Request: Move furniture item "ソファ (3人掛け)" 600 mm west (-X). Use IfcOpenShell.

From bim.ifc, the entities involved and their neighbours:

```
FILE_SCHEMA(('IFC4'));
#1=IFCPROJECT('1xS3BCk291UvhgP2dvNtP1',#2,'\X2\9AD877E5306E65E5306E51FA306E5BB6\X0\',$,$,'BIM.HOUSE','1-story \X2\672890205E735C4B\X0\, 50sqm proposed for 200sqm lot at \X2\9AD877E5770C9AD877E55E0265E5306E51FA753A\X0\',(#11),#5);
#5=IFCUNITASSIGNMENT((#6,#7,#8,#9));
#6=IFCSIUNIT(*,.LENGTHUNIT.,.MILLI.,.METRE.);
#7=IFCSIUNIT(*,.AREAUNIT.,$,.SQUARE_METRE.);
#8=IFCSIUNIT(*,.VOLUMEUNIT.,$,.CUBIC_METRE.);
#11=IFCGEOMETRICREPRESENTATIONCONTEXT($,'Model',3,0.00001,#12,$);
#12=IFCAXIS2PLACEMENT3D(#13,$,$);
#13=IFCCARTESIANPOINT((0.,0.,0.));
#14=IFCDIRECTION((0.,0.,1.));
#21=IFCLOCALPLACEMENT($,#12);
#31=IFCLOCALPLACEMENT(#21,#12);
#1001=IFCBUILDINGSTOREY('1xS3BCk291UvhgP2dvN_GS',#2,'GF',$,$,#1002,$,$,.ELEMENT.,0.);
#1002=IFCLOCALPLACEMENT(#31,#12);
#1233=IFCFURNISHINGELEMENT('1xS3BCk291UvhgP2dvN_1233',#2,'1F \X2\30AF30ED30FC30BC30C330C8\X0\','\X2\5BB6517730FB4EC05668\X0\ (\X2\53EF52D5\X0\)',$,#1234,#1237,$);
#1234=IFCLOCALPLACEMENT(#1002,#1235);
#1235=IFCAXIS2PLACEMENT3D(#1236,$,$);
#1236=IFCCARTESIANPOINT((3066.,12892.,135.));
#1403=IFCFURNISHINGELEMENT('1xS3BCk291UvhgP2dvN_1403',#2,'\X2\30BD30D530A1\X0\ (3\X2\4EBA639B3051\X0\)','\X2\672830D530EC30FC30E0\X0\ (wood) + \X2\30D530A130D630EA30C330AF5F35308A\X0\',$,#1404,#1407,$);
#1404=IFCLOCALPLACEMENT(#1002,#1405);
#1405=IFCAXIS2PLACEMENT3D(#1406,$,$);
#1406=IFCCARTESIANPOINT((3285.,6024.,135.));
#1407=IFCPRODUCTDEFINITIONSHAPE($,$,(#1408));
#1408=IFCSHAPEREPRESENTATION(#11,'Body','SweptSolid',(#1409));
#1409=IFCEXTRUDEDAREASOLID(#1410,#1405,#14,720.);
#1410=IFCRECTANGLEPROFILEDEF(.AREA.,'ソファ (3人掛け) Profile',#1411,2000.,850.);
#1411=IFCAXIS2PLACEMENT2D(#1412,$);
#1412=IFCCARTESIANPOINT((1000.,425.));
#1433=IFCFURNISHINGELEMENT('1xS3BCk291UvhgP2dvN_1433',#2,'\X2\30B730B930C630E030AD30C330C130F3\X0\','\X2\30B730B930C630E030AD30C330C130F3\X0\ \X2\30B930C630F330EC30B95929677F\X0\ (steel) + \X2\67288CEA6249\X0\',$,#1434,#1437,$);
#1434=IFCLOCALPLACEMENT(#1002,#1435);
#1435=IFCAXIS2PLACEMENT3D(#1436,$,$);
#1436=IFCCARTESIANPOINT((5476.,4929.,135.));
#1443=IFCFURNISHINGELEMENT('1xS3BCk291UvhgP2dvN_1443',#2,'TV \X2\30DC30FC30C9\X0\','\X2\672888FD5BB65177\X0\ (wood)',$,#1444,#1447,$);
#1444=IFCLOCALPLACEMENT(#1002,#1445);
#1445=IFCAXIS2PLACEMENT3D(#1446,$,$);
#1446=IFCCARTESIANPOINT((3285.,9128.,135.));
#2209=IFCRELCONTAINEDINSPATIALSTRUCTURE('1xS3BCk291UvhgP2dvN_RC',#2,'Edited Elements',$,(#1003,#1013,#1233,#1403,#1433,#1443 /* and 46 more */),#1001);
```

```python
import ifcopenshell
import ifcopenshell.api.geometry
import ifcopenshell.util.placement
import ifcopenshell.util.unit

model = ifcopenshell.open("bim.ifc")
unit_scale = ifcopenshell.util.unit.calculate_unit_scale(model)

item = model.by_id(1403)
matrix = ifcopenshell.util.placement.get_local_placement(item.ObjectPlacement)
matrix[0, 3] -= 0.6 / unit_scale
ifcopenshell.api.geometry.edit_object_placement(model, product=item, matrix=matrix, is_si=False)

print(ifcopenshell.util.placement.get_local_placement(item.ObjectPlacement).round(3) + 0.0)

model.write("bim-out.ifc")
```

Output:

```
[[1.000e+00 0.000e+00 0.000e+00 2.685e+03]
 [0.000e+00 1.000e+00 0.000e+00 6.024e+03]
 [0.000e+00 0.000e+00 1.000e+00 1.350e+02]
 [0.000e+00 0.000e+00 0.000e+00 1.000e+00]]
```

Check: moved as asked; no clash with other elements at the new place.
